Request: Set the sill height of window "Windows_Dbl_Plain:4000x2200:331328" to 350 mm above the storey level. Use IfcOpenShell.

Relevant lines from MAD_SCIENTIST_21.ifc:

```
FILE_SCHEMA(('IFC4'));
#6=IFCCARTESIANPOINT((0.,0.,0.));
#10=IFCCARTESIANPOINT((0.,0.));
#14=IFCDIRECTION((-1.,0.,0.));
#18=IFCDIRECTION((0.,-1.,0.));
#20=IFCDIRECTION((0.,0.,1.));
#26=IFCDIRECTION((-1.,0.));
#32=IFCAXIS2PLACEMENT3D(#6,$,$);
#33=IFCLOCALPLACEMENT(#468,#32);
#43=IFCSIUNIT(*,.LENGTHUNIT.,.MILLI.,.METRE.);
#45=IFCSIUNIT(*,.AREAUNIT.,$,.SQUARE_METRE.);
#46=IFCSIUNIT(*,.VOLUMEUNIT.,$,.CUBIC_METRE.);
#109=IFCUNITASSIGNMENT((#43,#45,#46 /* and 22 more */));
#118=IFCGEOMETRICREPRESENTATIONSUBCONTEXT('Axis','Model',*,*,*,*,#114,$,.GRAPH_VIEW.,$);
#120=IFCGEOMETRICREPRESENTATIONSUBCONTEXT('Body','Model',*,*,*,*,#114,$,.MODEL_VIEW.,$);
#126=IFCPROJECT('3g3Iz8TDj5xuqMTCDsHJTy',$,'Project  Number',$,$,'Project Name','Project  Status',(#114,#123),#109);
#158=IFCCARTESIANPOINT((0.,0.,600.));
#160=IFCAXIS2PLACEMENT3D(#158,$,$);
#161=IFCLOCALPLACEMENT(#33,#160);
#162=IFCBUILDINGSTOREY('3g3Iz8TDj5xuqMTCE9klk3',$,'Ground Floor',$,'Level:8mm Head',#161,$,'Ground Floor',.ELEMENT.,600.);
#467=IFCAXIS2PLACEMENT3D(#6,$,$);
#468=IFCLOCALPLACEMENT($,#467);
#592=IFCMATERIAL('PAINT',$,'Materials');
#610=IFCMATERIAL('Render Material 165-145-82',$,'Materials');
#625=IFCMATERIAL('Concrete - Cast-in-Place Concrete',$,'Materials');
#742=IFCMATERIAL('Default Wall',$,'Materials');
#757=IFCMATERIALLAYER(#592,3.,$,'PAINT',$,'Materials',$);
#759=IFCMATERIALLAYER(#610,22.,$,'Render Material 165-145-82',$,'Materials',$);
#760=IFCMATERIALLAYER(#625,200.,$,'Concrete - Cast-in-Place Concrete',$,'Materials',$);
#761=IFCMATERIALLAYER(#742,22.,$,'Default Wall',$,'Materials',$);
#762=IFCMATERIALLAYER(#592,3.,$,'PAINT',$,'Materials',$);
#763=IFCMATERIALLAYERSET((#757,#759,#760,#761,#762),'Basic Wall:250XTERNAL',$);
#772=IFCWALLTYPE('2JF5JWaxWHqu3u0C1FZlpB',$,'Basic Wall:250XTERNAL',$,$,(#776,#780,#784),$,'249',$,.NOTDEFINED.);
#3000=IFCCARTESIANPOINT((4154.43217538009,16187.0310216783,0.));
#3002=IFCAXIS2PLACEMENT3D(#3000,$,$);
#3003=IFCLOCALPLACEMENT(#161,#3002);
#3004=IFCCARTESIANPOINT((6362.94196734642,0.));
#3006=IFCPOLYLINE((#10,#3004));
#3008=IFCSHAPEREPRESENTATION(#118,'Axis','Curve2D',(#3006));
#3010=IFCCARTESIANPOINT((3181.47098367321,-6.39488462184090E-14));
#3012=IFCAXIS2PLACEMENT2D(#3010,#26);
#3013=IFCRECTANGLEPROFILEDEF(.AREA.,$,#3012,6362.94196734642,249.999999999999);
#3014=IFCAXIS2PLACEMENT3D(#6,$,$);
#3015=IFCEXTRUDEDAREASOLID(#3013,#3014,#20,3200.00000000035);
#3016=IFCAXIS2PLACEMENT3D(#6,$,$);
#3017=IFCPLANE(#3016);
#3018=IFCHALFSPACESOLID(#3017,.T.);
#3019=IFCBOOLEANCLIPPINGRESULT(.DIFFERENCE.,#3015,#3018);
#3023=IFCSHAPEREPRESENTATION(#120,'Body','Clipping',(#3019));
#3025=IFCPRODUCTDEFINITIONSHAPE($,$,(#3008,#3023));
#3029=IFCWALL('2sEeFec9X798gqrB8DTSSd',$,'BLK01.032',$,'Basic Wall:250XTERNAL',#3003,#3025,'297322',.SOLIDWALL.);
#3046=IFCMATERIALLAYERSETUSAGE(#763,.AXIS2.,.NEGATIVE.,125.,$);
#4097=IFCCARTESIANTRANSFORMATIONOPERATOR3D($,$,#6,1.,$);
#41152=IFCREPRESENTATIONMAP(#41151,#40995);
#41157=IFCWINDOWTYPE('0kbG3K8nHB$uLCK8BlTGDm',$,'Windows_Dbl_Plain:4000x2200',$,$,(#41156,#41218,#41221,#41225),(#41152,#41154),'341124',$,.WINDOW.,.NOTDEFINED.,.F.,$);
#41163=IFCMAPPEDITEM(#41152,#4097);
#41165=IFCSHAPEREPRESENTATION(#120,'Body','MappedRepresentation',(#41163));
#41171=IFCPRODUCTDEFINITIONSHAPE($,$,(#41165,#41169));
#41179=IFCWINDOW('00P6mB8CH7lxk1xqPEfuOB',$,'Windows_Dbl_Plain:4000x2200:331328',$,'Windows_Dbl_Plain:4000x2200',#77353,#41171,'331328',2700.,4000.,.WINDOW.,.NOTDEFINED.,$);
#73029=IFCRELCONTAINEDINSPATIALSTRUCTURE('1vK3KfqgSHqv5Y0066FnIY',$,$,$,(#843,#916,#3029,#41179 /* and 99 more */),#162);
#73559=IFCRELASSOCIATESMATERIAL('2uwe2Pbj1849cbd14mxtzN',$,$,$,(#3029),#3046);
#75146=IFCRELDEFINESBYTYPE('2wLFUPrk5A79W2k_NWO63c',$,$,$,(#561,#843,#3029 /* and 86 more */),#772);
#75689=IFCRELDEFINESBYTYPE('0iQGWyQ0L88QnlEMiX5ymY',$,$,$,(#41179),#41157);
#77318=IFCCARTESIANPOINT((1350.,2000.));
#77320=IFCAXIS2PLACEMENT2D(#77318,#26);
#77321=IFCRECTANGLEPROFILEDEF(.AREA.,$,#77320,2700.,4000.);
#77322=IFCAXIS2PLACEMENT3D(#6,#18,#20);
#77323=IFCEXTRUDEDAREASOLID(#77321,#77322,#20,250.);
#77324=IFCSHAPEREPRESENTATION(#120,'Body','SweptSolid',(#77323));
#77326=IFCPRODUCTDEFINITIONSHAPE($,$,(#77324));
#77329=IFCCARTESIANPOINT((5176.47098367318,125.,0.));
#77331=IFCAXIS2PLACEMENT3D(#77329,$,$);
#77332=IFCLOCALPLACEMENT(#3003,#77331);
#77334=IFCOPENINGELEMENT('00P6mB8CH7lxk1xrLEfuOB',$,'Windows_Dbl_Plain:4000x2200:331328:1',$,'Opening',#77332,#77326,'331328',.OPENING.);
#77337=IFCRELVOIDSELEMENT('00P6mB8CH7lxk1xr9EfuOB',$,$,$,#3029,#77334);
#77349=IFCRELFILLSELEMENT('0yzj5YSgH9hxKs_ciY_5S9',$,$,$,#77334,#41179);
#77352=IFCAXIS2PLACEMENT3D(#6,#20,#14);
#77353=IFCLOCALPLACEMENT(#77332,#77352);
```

```python
import numpy as np
import ifcopenshell
import ifcopenshell.api.geometry
import ifcopenshell.geom
import ifcopenshell.util.element
import ifcopenshell.util.placement
import ifcopenshell.util.shape
import ifcopenshell.util.unit

model = ifcopenshell.open("MAD_SCIENTIST_21.ifc")
unit_scale = ifcopenshell.util.unit.calculate_unit_scale(model)

window = model.by_guid("00P6mB8CH7lxk1xqPEfuOB")
opening = window.FillsVoids[0].RelatingOpeningElement
storey = ifcopenshell.util.element.get_container(window, ifc_class="IfcBuildingStorey")
level = ifcopenshell.util.placement.get_local_placement(storey.ObjectPlacement)[2, 3]

# The opening's origin need not be at the sill, so measure its lowest point.
shape = ifcopenshell.geom.create_shape(ifcopenshell.geom.settings(), opening)
bottom = ifcopenshell.util.shape.get_shape_bottom_elevation(shape, shape.geometry) / unit_scale
dz = level + 0.35 / unit_scale - bottom

shift = np.array([0.0, 0.0, dz])
# The window is placed relative to its opening, so it follows when the opening moves.
matrix = ifcopenshell.util.placement.get_local_placement(opening.ObjectPlacement)
matrix[:3, 3] += shift
ifcopenshell.api.geometry.edit_object_placement(
    model, product=opening, matrix=matrix, is_si=False, should_transform_children=True
)

print(f"moved by {dz * unit_scale:+.3f} m")

model.write("MAD_SCIENTIST_21-out.ifc")
```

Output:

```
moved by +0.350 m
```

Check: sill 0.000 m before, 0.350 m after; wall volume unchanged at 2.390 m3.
